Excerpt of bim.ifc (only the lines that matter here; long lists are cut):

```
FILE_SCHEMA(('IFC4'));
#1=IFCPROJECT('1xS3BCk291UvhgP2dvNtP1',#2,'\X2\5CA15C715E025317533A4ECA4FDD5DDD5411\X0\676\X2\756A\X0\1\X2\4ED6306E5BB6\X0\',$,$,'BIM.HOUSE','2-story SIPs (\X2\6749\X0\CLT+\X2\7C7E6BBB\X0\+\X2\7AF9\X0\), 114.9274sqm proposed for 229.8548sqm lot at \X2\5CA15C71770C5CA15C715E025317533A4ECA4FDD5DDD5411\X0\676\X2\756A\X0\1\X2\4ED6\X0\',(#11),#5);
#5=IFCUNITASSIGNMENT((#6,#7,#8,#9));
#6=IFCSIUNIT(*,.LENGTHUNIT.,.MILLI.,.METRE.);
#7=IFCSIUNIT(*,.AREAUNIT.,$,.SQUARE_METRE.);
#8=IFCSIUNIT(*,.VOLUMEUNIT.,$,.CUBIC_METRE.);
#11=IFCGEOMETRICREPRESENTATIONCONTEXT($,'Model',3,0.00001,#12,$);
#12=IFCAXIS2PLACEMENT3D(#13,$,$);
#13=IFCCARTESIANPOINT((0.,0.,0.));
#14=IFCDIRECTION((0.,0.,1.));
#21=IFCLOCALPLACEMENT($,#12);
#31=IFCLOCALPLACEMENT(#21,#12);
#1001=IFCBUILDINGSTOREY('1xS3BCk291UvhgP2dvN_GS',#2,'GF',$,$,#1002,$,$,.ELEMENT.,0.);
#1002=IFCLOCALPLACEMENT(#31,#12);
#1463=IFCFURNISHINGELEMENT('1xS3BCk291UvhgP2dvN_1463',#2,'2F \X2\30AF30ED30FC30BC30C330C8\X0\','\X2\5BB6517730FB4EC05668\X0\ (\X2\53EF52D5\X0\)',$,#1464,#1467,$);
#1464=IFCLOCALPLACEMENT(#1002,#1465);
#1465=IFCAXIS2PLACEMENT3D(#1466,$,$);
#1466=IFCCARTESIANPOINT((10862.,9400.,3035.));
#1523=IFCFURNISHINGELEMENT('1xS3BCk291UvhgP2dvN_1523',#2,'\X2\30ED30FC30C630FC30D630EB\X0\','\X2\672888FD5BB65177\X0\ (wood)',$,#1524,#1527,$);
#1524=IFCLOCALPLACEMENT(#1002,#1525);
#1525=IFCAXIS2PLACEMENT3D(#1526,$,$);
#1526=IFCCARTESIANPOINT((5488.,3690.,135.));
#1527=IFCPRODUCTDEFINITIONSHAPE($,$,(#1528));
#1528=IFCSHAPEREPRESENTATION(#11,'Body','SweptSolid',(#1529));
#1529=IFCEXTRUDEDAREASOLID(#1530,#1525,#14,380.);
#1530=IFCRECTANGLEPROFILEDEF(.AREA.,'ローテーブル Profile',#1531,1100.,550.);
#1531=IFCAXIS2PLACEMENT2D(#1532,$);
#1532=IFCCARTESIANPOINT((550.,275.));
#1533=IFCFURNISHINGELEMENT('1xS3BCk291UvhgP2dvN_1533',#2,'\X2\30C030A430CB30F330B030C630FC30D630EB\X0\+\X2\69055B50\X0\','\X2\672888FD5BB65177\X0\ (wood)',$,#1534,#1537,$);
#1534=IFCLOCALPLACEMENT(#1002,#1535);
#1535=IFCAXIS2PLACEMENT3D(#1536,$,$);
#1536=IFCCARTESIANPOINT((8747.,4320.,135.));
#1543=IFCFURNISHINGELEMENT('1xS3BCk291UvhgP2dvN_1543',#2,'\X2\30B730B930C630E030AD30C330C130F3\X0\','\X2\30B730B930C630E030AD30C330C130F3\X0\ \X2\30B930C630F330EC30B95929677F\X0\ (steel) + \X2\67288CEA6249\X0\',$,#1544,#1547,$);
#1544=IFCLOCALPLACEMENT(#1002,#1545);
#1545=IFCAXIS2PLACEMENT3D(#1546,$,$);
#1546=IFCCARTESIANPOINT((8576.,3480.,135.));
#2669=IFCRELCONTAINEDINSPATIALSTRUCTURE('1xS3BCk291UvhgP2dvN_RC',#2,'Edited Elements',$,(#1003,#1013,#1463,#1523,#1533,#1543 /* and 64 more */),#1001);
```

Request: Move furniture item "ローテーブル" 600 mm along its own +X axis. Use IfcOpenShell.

```python
import ifcopenshell
import ifcopenshell.api.geometry
import ifcopenshell.util.placement

model = ifcopenshell.open("bim.ifc")

item = model.by_guid("1xS3BCk291UvhgP2dvN_1523")
matrix = ifcopenshell.util.placement.get_local_placement(item.ObjectPlacement)
matrix[:3, 3] += matrix[:3, 0] * 600.0
ifcopenshell.api.geometry.edit_object_placement(model, product=item, matrix=matrix, is_si=False)

print(ifcopenshell.util.placement.get_local_placement(item.ObjectPlacement).round(3) + 0.0)

model.write("bim_v2.ifc")
```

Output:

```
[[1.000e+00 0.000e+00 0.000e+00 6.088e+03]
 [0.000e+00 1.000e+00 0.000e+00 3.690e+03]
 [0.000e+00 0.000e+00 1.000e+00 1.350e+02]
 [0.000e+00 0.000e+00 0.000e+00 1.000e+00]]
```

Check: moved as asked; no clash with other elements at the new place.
